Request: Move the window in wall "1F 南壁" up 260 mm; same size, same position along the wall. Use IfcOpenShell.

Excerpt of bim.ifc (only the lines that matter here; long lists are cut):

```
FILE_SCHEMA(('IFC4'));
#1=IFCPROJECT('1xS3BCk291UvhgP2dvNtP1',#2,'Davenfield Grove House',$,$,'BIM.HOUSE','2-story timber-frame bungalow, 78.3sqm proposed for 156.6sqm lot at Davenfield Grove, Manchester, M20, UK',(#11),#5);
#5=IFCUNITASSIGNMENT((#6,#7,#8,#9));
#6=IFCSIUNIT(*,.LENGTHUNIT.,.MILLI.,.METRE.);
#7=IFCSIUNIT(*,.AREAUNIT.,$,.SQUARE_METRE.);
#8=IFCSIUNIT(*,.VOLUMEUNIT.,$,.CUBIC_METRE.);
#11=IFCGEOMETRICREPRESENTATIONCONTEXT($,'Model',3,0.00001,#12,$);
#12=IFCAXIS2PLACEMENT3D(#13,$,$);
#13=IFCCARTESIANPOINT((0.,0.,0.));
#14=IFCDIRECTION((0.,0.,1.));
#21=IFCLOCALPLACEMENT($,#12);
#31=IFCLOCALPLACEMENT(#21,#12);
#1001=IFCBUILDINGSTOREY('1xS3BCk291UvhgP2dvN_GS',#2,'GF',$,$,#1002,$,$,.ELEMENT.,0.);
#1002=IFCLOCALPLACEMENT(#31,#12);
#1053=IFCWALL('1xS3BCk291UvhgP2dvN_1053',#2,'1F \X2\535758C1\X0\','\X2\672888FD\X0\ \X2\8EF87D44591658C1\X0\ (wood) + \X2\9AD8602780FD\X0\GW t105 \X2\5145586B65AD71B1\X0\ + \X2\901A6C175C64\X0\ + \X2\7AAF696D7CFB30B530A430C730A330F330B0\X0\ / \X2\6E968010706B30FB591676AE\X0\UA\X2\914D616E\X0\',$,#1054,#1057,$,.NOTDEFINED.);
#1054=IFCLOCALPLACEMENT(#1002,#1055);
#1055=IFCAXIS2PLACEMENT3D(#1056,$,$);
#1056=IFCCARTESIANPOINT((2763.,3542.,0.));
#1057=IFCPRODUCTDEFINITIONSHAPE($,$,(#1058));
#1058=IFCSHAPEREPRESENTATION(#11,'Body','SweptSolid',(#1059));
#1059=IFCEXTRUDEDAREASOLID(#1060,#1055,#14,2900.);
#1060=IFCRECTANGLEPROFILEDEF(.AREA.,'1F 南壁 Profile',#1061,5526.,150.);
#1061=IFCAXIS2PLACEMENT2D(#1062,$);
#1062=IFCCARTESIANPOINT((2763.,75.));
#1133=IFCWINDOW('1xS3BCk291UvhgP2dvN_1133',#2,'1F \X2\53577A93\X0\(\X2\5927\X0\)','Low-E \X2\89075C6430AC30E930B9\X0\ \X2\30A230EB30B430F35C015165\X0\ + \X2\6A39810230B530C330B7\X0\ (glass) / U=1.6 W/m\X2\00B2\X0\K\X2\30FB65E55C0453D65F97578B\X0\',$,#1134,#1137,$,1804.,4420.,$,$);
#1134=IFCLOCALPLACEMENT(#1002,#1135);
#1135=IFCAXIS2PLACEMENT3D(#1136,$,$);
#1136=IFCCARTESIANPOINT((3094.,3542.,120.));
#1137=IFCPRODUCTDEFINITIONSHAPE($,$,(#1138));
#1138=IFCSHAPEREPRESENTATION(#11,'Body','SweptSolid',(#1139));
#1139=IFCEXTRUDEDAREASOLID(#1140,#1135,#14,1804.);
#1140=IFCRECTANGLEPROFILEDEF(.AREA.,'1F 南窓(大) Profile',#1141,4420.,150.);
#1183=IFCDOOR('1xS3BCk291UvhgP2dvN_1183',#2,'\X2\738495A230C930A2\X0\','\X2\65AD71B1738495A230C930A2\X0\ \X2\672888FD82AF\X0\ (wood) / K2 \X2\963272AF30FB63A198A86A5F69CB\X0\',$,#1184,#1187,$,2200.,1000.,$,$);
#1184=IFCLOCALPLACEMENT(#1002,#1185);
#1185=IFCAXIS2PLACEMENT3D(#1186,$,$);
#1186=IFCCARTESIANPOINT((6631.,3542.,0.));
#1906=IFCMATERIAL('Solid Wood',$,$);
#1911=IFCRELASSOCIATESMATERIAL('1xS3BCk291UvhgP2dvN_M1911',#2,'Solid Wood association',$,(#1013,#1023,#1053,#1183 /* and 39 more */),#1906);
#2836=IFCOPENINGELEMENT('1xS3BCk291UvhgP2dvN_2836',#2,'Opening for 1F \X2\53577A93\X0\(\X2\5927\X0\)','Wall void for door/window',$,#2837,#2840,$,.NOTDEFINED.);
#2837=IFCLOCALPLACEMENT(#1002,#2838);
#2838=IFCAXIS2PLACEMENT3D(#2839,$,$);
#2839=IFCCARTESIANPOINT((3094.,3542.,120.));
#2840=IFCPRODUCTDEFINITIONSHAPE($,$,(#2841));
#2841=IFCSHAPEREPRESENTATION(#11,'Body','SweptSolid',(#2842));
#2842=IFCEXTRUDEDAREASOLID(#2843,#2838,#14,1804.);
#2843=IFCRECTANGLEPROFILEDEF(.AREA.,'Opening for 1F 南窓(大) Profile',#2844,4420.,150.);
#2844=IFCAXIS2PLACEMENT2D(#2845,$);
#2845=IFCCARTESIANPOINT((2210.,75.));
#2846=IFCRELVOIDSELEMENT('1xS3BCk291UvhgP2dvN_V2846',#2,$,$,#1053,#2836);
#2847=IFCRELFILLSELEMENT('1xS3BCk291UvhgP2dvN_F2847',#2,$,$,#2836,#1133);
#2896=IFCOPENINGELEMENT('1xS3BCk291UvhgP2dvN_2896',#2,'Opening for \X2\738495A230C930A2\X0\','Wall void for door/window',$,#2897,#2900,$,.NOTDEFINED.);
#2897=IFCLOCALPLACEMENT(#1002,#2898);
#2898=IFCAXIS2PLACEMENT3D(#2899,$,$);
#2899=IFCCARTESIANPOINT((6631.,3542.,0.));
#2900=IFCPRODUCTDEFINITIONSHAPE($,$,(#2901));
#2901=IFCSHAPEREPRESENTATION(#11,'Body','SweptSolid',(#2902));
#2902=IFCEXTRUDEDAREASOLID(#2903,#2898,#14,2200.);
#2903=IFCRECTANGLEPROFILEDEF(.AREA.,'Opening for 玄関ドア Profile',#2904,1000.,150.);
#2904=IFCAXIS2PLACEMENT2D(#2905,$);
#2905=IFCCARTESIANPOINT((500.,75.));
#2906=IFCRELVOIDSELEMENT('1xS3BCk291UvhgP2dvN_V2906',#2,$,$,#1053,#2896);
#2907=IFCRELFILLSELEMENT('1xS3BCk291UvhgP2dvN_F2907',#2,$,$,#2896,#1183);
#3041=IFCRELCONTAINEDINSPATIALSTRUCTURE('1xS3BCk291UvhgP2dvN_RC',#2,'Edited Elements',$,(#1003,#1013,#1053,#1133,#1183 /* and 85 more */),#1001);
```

```python
import numpy as np
import ifcopenshell
import ifcopenshell.api.geometry
import ifcopenshell.util.placement
import ifcopenshell.util.unit

model = ifcopenshell.open("bim.ifc")
unit_scale = ifcopenshell.util.unit.calculate_unit_scale(model)

window = model.by_guid("1xS3BCk291UvhgP2dvN_1133")
opening = window.FillsVoids[0].RelatingOpeningElement
dz = 0.26 / unit_scale

shift = np.array([0.0, 0.0, dz])
# The window is not placed relative to its opening, so move both.
for product in (opening, window):
    matrix = ifcopenshell.util.placement.get_local_placement(product.ObjectPlacement)
    matrix[:3, 3] += shift
    ifcopenshell.api.geometry.edit_object_placement(model, product=product, matrix=matrix, is_si=False)

print(f"moved by {dz * unit_scale:+.3f} m")

model.write("bim_updated.ifc")
```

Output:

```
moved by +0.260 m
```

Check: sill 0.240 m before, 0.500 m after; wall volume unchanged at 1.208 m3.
